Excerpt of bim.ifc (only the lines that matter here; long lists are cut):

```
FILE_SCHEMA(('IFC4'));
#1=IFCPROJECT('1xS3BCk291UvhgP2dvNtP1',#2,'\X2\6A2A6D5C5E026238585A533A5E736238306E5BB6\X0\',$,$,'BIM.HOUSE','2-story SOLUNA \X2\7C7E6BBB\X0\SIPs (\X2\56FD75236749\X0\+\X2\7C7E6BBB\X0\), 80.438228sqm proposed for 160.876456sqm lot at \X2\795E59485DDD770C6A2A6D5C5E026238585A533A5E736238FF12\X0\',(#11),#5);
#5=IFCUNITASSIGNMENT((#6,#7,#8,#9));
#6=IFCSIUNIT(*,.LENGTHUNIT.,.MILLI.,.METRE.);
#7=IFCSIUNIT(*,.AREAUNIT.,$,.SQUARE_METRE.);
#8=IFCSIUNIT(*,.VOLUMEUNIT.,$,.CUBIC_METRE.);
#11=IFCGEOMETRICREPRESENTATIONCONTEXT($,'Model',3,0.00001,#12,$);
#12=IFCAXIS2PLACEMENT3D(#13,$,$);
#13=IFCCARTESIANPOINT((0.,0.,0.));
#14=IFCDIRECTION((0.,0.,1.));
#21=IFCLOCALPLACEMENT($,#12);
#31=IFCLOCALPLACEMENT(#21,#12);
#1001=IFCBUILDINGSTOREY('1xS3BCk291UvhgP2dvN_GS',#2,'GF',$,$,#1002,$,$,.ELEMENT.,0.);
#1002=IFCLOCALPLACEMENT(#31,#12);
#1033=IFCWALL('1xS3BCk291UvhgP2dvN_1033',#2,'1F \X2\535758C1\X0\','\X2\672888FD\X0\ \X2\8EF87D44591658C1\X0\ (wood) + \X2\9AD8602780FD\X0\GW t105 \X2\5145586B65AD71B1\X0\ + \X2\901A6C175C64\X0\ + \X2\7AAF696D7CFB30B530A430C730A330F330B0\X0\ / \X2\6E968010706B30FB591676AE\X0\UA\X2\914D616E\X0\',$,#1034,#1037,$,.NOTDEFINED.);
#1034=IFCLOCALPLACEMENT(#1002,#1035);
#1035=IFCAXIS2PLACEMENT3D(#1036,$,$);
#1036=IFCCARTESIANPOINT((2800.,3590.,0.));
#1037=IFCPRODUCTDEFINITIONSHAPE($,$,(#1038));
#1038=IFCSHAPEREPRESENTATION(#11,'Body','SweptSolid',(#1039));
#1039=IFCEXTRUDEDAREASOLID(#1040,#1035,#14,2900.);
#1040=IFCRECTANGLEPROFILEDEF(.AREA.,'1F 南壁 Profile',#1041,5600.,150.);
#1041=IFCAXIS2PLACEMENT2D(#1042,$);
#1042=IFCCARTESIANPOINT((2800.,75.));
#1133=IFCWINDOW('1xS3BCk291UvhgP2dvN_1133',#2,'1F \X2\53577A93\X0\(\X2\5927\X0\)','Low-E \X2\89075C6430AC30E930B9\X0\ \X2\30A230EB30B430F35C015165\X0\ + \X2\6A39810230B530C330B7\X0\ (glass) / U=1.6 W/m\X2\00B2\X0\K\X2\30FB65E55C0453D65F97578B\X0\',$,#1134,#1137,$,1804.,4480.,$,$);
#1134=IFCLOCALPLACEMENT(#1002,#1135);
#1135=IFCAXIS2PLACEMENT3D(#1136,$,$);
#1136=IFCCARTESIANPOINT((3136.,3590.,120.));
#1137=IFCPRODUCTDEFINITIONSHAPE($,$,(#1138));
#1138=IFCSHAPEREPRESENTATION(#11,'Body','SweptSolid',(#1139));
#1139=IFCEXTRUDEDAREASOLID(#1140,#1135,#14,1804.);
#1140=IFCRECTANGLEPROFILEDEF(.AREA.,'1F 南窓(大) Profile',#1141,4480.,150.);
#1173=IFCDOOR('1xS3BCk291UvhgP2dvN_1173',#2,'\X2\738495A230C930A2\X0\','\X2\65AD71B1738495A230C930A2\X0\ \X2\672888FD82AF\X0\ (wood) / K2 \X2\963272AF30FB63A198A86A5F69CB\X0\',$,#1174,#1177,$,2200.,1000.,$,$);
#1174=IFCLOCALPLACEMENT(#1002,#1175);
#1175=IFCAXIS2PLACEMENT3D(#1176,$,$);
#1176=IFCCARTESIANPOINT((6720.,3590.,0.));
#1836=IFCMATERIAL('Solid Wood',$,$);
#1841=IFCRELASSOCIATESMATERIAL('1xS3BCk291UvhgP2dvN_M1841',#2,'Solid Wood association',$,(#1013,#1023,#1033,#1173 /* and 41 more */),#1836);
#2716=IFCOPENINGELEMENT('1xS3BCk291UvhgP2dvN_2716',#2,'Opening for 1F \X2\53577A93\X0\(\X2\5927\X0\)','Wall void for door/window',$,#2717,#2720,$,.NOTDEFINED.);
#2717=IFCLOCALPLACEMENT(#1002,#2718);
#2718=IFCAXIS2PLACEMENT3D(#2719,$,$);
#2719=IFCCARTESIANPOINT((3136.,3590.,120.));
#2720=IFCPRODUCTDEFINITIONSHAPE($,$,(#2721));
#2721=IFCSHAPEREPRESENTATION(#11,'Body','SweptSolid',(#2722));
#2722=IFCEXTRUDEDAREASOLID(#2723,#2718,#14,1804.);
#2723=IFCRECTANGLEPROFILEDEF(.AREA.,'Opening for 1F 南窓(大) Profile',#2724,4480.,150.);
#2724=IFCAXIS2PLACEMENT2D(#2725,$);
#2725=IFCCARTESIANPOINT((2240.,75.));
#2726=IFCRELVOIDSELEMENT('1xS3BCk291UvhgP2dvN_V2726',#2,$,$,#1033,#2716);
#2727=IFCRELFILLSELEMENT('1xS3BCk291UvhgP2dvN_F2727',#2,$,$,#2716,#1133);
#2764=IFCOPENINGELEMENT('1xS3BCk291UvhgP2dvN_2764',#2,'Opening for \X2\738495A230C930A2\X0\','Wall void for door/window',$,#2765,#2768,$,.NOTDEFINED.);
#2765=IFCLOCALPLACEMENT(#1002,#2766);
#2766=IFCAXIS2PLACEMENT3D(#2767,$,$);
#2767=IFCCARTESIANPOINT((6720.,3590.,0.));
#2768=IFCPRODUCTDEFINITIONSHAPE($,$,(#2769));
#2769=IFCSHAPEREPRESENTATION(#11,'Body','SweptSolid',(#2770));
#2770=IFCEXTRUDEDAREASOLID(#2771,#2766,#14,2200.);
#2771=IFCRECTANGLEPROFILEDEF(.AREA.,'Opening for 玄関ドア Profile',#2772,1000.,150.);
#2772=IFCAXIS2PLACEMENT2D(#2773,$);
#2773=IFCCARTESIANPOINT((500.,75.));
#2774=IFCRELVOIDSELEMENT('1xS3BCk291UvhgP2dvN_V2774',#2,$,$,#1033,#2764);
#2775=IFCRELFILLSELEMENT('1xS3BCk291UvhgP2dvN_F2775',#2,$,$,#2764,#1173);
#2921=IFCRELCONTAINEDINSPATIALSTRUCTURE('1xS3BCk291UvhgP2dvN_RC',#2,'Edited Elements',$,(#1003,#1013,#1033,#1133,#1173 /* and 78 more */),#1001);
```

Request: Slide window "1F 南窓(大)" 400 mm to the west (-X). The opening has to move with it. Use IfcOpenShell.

```python
import ifcopenshell
import ifcopenshell.api.geometry
import ifcopenshell.util.placement
import ifcopenshell.util.unit

model = ifcopenshell.open("bim.ifc")
unit_scale = ifcopenshell.util.unit.calculate_unit_scale(model)

window = model.by_guid("1xS3BCk291UvhgP2dvN_1133")
opening = window.FillsVoids[0].RelatingOpeningElement
wall = opening.VoidsElements[0].RelatingBuildingElement

wall_matrix = ifcopenshell.util.placement.get_local_placement(wall.ObjectPlacement)
shift = wall_matrix[:3, 0] * -0.4 / unit_scale
before = ifcopenshell.util.placement.get_local_placement(window.ObjectPlacement)[:3, 3].copy()

# The window is not placed relative to its opening, so move both.
for product in (opening, window):
    matrix = ifcopenshell.util.placement.get_local_placement(product.ObjectPlacement)
    matrix[:3, 3] += shift
    ifcopenshell.api.geometry.edit_object_placement(model, product=product, matrix=matrix, is_si=False)

after = ifcopenshell.util.placement.get_local_placement(window.ObjectPlacement)[:3, 3]
print("window moved by", (after - before).round(3) + 0.0)

model.write("bim_updated.ifc")
```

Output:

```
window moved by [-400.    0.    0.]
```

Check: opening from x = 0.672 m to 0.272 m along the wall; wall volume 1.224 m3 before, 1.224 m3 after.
